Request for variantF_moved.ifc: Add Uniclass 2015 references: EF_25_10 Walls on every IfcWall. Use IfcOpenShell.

First a look at what the model holds.

```python
import ifcopenshell

model = ifcopenshell.open("variantF_moved.ifc")
print(model.schema)
print("classifications:", [c.Name for c in model.by_type("IfcClassification")])
for ifc_class in ("IfcDoor", "IfcRoof", "IfcStair", "IfcWall", "IfcWindow"):
    print(ifc_class, len(model.by_type(ifc_class)))
```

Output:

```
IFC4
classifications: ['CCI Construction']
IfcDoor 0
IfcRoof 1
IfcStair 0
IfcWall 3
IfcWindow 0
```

```python
import ifcopenshell
import ifcopenshell.api.classification

model = ifcopenshell.open("variantF_moved.ifc")

system = ifcopenshell.api.classification.add_classification(model, classification="Uniclass 2015")

codes = {
    "IfcWall": ("EF_25_10", "Walls"),
}
for ifc_class, (code, name) in codes.items():
    products = model.by_type(ifc_class)
    ifcopenshell.api.classification.add_reference(
        model, products=products, classification=system, identification=code, name=name
    )
    print(code, len(products))

model.write("variantF_moved_v2.ifc")
```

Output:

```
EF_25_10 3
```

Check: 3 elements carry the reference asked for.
